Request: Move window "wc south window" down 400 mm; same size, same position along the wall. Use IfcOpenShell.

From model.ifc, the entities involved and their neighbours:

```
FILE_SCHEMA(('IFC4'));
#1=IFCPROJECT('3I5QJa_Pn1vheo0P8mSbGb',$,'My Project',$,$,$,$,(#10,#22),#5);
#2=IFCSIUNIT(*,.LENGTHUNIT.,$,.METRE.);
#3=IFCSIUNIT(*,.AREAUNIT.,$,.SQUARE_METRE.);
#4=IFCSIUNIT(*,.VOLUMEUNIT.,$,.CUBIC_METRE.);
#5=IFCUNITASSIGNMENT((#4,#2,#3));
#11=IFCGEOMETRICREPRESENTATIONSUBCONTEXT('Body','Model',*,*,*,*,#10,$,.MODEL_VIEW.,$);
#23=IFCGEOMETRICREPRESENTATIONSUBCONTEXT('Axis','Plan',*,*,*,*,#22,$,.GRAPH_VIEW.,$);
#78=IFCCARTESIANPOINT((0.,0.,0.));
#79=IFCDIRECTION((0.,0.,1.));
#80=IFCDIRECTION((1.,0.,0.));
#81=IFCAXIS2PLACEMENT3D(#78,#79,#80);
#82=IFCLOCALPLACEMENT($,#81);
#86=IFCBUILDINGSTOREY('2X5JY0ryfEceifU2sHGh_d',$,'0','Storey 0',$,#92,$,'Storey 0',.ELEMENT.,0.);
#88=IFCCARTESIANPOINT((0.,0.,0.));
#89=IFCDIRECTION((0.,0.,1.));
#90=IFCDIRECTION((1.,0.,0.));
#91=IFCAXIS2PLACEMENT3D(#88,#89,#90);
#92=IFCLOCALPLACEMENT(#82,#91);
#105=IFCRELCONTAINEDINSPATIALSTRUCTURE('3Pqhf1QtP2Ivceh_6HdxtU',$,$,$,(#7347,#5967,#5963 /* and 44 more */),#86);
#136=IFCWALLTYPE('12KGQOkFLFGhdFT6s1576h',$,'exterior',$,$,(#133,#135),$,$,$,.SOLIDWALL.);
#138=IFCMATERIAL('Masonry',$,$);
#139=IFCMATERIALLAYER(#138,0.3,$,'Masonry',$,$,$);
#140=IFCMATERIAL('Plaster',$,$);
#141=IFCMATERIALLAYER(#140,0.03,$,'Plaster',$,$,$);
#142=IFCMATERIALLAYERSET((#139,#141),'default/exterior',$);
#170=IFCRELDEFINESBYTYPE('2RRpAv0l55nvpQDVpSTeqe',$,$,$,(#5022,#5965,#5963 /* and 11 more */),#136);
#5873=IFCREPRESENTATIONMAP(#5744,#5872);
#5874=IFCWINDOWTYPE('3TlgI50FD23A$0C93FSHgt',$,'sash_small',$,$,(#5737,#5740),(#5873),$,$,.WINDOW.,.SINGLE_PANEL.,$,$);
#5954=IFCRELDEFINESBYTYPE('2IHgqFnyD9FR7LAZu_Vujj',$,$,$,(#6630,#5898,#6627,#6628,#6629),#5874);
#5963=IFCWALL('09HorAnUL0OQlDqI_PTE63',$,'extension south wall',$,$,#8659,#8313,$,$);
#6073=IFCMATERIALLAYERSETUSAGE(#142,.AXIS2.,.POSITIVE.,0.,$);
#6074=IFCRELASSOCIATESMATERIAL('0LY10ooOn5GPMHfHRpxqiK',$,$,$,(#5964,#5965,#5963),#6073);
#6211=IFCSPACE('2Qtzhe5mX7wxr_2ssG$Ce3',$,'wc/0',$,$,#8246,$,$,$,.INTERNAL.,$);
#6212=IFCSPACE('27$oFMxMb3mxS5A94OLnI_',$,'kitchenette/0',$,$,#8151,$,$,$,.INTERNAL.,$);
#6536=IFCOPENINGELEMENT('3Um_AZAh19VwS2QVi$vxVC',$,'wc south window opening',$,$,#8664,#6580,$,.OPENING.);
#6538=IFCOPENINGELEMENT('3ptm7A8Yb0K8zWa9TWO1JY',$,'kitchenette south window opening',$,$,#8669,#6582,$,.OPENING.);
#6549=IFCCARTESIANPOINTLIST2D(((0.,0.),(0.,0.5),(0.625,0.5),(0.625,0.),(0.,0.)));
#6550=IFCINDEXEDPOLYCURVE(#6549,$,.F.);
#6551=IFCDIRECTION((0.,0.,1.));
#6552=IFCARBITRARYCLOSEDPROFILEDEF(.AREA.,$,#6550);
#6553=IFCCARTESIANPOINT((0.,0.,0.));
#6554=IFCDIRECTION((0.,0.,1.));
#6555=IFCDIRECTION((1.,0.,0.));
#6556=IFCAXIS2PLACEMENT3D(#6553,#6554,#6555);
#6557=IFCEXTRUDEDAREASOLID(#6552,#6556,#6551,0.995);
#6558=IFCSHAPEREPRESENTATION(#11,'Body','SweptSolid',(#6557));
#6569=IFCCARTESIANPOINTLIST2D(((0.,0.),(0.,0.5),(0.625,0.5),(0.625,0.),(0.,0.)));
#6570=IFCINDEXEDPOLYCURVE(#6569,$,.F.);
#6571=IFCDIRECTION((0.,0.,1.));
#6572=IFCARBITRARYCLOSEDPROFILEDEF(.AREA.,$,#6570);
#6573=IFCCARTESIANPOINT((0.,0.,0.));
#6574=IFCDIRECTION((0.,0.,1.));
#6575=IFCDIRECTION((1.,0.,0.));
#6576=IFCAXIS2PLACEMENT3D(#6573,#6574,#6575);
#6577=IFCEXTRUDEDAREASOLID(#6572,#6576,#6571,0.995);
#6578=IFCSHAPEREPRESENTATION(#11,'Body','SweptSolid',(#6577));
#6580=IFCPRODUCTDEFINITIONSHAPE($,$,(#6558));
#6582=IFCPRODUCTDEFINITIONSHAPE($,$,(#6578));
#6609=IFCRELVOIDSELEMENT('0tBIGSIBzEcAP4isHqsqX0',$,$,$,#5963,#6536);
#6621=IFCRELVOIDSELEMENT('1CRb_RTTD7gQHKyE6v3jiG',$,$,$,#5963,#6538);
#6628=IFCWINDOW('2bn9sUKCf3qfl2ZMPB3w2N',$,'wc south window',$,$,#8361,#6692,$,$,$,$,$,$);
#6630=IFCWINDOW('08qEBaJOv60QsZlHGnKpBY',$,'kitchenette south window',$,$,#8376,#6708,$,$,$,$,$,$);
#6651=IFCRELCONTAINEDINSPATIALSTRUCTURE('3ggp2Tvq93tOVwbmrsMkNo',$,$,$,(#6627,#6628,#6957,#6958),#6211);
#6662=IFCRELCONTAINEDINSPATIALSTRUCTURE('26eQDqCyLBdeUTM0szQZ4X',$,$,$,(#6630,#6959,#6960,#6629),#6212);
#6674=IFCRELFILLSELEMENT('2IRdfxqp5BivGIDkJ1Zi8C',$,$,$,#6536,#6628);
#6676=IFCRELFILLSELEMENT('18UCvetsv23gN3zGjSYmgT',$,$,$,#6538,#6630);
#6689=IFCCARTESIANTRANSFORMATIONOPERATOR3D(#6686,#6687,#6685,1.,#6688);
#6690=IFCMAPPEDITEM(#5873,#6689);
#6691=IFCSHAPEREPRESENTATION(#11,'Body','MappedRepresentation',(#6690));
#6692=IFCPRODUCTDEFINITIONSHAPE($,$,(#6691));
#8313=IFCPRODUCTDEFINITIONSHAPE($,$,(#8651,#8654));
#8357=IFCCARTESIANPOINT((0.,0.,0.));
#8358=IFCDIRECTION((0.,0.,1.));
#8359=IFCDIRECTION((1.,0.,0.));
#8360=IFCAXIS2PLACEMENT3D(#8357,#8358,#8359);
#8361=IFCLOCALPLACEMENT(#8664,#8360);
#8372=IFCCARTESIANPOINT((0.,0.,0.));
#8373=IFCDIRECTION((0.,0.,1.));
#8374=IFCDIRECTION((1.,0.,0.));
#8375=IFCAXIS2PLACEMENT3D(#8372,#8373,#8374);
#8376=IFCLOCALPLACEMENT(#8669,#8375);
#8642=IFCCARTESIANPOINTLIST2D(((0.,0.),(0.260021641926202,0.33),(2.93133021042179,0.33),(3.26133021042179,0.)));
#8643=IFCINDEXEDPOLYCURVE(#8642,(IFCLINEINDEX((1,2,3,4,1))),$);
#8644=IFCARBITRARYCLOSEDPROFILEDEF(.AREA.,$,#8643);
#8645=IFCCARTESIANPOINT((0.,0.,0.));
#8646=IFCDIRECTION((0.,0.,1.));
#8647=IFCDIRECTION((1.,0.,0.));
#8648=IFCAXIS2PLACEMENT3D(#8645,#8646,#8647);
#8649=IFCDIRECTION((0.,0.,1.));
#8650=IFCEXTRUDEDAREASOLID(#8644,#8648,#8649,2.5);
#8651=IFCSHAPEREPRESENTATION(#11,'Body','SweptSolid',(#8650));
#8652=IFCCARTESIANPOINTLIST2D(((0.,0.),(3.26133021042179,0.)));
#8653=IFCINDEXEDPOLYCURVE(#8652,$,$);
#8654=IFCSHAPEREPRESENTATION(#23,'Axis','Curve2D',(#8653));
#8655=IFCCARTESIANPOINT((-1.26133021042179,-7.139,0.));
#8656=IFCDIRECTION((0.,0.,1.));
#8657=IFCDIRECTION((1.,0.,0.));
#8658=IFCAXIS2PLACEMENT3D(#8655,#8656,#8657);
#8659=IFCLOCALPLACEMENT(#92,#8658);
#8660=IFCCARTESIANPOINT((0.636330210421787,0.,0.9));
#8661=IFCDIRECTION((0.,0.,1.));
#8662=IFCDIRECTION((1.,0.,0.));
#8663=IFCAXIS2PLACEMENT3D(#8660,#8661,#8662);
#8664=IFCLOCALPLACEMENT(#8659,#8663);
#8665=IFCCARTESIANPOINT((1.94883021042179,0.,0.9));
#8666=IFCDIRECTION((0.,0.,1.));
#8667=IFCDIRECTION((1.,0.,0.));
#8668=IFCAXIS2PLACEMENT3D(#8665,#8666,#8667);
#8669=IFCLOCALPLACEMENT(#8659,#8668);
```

```python
import numpy as np
import ifcopenshell
import ifcopenshell.api.geometry
import ifcopenshell.util.placement
import ifcopenshell.util.unit

model = ifcopenshell.open("model.ifc")
unit_scale = ifcopenshell.util.unit.calculate_unit_scale(model)

window = model.by_guid("2bn9sUKCf3qfl2ZMPB3w2N")
opening = window.FillsVoids[0].RelatingOpeningElement
dz = -0.4

shift = np.array([0.0, 0.0, dz])
# The window is placed relative to its opening, so it follows when the opening moves.
matrix = ifcopenshell.util.placement.get_local_placement(opening.ObjectPlacement)
matrix[:3, 3] += shift
ifcopenshell.api.geometry.edit_object_placement(
    model, product=opening, matrix=matrix, is_si=False, should_transform_children=True
)

print(f"moved by {dz * unit_scale:+.3f} m")

model.write("model_updated.ifc")
```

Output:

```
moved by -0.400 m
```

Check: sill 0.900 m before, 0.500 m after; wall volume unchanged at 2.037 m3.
